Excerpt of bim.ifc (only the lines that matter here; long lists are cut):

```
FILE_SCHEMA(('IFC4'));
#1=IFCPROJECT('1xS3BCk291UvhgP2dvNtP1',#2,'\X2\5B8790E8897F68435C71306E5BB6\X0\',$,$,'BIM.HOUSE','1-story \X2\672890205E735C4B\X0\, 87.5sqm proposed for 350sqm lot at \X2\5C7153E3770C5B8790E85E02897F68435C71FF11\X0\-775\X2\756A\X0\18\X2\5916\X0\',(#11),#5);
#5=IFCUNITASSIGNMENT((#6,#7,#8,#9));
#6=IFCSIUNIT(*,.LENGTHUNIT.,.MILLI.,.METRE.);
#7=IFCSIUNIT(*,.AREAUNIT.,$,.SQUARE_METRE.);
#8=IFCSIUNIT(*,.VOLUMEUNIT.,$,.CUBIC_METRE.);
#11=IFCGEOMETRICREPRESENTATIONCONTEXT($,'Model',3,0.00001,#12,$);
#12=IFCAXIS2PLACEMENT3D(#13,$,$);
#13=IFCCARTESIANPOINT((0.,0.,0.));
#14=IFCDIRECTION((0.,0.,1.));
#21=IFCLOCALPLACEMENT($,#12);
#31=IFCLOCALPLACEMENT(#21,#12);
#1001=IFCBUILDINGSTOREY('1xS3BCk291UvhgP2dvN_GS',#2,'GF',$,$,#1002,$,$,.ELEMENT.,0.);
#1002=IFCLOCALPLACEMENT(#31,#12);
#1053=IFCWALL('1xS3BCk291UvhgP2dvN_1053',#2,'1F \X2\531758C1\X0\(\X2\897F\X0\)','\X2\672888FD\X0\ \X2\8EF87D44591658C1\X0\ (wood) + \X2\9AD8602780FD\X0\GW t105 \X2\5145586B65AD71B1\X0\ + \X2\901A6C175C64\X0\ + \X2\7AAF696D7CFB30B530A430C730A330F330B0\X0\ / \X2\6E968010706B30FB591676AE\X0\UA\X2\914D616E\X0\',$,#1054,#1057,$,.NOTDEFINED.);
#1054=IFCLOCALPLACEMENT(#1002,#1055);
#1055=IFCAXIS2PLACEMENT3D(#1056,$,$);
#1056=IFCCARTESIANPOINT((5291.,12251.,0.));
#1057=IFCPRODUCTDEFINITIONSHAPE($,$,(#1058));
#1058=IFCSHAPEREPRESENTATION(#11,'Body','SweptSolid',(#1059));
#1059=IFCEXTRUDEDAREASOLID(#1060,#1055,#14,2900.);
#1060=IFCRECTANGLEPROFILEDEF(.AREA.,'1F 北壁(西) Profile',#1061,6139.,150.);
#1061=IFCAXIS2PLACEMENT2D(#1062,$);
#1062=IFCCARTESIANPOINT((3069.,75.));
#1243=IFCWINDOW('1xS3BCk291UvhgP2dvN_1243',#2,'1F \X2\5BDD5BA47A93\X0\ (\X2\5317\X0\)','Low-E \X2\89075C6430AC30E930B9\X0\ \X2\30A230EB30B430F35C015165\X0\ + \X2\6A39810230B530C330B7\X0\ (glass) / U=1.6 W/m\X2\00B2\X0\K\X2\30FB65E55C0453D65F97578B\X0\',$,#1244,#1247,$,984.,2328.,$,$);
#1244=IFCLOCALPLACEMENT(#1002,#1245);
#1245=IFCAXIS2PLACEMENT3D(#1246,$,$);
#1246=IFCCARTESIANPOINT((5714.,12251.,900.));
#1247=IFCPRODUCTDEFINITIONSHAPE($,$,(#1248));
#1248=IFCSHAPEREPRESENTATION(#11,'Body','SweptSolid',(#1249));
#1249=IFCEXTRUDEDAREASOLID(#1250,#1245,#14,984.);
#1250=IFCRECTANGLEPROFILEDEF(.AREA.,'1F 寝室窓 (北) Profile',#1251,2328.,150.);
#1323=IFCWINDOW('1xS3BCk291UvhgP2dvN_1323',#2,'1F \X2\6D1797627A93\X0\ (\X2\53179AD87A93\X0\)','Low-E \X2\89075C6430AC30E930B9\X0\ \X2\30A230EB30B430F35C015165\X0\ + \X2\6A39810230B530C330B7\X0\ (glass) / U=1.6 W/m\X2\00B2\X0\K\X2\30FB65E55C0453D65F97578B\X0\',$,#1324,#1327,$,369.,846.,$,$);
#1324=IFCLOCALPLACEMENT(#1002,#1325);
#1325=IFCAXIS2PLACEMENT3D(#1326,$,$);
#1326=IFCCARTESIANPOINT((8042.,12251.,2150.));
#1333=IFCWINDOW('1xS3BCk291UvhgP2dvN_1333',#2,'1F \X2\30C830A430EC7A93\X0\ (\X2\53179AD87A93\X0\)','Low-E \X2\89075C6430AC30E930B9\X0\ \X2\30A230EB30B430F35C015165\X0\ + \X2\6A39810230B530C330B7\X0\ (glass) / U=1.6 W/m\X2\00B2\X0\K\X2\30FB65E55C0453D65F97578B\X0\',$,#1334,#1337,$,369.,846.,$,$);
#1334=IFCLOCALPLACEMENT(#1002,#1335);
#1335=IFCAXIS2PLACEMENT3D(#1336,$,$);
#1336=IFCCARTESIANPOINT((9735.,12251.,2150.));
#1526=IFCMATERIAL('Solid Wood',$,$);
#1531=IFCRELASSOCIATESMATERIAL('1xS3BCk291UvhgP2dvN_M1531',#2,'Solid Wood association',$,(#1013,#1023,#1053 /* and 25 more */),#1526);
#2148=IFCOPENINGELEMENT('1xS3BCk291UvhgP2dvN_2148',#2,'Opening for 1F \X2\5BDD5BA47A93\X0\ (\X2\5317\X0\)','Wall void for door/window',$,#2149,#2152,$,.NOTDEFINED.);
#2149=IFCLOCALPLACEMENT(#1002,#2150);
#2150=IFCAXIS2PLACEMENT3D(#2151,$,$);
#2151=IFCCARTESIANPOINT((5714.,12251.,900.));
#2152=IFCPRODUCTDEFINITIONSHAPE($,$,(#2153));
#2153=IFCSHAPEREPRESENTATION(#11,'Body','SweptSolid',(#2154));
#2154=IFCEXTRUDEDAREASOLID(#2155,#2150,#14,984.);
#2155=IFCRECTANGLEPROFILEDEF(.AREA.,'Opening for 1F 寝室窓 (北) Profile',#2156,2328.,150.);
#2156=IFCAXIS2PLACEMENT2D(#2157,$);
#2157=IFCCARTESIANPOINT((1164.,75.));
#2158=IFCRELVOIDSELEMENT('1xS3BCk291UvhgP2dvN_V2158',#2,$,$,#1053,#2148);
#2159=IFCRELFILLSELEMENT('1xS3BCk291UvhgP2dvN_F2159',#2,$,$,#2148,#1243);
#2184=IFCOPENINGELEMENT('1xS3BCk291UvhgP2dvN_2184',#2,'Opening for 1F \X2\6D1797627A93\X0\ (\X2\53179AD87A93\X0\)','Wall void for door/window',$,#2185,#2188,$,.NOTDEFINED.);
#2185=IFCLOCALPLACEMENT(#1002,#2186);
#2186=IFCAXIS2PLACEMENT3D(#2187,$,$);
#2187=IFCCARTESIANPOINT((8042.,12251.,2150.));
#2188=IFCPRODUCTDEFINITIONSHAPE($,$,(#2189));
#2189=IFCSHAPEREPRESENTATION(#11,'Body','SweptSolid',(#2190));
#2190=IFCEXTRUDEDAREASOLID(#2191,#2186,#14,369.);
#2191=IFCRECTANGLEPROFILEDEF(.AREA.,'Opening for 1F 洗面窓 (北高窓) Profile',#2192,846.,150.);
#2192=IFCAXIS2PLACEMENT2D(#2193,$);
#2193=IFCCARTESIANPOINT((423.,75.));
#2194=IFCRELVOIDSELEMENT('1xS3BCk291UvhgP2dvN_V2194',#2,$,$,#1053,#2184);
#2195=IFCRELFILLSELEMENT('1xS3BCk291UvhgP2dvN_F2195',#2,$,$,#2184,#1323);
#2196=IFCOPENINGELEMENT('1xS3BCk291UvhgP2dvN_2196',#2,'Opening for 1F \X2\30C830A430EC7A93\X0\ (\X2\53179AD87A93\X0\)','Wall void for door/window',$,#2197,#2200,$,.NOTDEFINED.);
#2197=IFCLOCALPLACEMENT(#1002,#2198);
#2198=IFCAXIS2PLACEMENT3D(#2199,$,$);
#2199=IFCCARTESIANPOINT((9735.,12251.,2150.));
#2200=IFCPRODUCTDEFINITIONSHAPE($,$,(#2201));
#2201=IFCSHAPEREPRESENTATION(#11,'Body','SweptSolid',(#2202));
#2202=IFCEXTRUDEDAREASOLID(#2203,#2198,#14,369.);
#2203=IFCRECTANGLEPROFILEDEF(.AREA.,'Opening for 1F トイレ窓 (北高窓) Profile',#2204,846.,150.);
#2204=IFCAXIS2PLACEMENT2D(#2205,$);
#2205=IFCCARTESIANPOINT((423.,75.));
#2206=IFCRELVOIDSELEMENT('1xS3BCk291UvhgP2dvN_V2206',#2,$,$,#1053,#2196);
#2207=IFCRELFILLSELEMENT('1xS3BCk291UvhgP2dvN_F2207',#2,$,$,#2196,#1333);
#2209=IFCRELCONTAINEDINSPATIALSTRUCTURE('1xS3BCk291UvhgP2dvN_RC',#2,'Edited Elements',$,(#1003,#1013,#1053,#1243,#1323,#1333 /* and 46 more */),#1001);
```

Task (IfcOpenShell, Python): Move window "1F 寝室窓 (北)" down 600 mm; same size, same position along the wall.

```python
import numpy as np
import ifcopenshell
import ifcopenshell.api.geometry
import ifcopenshell.util.placement
import ifcopenshell.util.unit

model = ifcopenshell.open("bim.ifc")
unit_scale = ifcopenshell.util.unit.calculate_unit_scale(model)

window = model.by_guid("1xS3BCk291UvhgP2dvN_1243")
opening = window.FillsVoids[0].RelatingOpeningElement
dz = -0.6 / unit_scale

shift = np.array([0.0, 0.0, dz])
# The window is not placed relative to its opening, so move both.
for product in (opening, window):
    matrix = ifcopenshell.util.placement.get_local_placement(product.ObjectPlacement)
    matrix[:3, 3] += shift
    ifcopenshell.api.geometry.edit_object_placement(model, product=product, matrix=matrix, is_si=False)

print(f"moved by {dz * unit_scale:+.3f} m")

model.write("bim-out.ifc")
```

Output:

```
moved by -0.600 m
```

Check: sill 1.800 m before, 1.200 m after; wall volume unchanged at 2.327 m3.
